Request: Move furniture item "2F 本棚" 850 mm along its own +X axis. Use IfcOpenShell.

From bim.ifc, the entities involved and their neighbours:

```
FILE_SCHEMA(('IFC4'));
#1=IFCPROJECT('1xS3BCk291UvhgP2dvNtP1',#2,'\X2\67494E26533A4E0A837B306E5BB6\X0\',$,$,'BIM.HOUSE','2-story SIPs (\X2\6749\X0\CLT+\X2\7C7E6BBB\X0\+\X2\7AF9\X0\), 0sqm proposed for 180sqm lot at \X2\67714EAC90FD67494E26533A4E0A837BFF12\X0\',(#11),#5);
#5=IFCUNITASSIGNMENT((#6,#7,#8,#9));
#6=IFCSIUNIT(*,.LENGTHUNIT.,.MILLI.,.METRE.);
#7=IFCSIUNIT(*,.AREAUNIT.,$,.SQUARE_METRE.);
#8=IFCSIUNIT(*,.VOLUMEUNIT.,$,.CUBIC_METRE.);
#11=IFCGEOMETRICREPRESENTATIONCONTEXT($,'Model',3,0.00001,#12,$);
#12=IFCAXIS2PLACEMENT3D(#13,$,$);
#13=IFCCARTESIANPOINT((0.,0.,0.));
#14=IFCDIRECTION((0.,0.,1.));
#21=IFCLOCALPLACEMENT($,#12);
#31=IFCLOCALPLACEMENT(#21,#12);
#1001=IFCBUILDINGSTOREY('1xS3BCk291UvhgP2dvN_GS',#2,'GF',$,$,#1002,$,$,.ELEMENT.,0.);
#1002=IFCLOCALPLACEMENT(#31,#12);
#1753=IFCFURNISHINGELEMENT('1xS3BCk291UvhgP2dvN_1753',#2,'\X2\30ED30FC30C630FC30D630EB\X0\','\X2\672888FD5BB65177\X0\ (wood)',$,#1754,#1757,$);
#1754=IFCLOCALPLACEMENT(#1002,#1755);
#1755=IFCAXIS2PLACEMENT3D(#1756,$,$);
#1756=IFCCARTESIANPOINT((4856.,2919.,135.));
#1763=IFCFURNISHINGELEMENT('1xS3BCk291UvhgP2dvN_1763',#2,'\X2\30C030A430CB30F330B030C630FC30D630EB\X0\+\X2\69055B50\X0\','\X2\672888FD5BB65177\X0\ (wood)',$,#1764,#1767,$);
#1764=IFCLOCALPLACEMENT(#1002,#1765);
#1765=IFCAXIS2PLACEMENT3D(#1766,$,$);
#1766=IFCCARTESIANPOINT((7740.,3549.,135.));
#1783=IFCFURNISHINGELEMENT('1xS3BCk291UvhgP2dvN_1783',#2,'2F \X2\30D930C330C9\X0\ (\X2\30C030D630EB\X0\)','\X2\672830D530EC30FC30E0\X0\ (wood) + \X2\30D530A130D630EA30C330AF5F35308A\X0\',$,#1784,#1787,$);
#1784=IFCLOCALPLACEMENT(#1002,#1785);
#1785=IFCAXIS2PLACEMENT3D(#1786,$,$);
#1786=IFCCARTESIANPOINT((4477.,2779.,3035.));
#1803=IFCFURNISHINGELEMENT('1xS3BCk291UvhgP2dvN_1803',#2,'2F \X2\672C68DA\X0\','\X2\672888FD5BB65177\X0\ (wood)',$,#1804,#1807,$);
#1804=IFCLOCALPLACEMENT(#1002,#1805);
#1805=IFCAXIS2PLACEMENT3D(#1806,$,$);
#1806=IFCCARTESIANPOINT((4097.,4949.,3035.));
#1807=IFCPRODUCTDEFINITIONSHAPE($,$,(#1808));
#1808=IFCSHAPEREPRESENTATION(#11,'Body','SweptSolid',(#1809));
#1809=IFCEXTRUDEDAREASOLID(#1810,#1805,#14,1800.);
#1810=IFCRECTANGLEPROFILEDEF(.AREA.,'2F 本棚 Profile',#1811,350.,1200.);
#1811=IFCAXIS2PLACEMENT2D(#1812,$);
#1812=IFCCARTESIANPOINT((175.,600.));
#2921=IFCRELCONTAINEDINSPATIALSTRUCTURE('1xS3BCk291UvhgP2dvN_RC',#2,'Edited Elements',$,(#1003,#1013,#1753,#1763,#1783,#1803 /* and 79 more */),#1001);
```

```python
import ifcopenshell
import ifcopenshell.api.geometry
import ifcopenshell.util.placement
import ifcopenshell.util.unit

model = ifcopenshell.open("bim.ifc")
unit_scale = ifcopenshell.util.unit.calculate_unit_scale(model)

item = model.by_guid("1xS3BCk291UvhgP2dvN_1803")
matrix = ifcopenshell.util.placement.get_local_placement(item.ObjectPlacement)
matrix[:3, 3] += matrix[:3, 0] * 0.85 / unit_scale
ifcopenshell.api.geometry.edit_object_placement(model, product=item, matrix=matrix, is_si=False)

print(ifcopenshell.util.placement.get_local_placement(item.ObjectPlacement).round(3) + 0.0)

model.write("bim_rev.ifc")
```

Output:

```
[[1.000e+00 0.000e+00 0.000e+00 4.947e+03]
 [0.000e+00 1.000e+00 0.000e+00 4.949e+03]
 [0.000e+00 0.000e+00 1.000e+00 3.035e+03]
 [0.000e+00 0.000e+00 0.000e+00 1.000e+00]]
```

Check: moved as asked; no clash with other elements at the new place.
